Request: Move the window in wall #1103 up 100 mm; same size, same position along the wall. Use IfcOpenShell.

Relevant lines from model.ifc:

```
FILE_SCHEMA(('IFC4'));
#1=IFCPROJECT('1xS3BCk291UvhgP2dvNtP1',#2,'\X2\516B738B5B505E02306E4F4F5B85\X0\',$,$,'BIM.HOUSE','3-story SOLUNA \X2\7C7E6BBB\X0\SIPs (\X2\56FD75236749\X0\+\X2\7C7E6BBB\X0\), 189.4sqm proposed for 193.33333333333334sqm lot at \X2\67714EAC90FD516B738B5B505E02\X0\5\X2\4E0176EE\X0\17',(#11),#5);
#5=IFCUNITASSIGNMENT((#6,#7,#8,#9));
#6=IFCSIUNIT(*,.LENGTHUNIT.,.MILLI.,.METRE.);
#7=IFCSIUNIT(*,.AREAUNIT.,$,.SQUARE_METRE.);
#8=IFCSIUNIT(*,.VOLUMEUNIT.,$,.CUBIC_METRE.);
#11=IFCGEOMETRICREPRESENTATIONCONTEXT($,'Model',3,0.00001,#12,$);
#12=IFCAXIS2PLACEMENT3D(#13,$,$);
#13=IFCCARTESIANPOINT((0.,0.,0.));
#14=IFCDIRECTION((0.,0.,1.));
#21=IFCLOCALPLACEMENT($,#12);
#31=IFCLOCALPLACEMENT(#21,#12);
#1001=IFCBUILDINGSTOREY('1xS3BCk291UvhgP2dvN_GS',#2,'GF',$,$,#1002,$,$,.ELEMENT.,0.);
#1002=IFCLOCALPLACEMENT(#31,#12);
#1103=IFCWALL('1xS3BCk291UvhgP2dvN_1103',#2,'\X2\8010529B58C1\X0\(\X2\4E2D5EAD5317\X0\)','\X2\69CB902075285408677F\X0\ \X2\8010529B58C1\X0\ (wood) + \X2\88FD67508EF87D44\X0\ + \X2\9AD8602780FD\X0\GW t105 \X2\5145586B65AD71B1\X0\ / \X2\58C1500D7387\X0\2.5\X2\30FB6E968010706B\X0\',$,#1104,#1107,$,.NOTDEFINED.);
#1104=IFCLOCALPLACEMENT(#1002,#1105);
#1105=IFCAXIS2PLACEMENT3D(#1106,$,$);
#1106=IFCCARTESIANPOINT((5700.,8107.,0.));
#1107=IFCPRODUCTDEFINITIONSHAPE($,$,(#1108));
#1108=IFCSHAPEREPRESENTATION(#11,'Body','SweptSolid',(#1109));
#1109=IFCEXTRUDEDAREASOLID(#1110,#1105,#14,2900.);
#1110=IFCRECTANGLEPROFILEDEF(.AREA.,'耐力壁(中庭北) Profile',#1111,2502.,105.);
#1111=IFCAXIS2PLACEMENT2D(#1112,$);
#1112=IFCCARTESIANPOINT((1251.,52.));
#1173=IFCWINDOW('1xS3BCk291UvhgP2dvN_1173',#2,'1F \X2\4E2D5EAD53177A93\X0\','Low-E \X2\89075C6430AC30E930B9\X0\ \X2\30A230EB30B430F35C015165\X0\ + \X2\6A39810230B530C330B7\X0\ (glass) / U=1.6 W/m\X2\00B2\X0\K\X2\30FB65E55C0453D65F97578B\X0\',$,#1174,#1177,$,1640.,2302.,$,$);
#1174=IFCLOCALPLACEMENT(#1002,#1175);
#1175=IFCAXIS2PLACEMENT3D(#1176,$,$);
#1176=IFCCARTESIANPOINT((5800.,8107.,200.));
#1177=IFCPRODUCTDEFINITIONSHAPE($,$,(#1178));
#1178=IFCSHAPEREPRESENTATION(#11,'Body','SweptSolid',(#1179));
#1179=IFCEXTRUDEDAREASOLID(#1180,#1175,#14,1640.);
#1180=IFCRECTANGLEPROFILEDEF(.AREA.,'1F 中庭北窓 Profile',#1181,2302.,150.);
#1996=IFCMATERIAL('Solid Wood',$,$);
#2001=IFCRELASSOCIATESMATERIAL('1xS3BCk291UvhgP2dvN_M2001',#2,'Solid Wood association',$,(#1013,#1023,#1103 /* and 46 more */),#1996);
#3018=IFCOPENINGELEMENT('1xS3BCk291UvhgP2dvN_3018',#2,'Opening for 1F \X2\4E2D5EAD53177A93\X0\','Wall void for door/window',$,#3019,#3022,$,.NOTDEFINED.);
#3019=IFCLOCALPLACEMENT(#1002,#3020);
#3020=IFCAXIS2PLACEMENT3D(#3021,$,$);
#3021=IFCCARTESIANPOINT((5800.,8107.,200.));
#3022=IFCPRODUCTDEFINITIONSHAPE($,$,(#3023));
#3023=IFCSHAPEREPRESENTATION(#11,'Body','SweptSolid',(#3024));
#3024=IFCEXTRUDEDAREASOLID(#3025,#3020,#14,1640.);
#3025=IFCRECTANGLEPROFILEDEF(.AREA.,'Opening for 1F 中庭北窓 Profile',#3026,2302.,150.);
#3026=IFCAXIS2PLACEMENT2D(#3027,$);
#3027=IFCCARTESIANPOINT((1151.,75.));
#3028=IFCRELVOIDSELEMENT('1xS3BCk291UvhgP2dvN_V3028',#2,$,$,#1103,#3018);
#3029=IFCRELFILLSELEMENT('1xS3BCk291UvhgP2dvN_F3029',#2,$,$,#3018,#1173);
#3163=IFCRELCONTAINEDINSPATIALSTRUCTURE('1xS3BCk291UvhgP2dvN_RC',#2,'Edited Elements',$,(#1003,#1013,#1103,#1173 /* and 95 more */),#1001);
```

```python
import numpy as np
import ifcopenshell
import ifcopenshell.api.geometry
import ifcopenshell.util.placement
import ifcopenshell.util.unit

model = ifcopenshell.open("model.ifc")
unit_scale = ifcopenshell.util.unit.calculate_unit_scale(model)

window = model.by_guid("1xS3BCk291UvhgP2dvN_1173")
opening = window.FillsVoids[0].RelatingOpeningElement
dz = 100.0

shift = np.array([0.0, 0.0, dz])
# The window is not placed relative to its opening, so move both.
for product in (opening, window):
    matrix = ifcopenshell.util.placement.get_local_placement(product.ObjectPlacement)
    matrix[:3, 3] += shift
    ifcopenshell.api.geometry.edit_object_placement(model, product=product, matrix=matrix, is_si=False)

print(f"moved by {dz * unit_scale:+.3f} m")

model.write("model-out.ifc")
```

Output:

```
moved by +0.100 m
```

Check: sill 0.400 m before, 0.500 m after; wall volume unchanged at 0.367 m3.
